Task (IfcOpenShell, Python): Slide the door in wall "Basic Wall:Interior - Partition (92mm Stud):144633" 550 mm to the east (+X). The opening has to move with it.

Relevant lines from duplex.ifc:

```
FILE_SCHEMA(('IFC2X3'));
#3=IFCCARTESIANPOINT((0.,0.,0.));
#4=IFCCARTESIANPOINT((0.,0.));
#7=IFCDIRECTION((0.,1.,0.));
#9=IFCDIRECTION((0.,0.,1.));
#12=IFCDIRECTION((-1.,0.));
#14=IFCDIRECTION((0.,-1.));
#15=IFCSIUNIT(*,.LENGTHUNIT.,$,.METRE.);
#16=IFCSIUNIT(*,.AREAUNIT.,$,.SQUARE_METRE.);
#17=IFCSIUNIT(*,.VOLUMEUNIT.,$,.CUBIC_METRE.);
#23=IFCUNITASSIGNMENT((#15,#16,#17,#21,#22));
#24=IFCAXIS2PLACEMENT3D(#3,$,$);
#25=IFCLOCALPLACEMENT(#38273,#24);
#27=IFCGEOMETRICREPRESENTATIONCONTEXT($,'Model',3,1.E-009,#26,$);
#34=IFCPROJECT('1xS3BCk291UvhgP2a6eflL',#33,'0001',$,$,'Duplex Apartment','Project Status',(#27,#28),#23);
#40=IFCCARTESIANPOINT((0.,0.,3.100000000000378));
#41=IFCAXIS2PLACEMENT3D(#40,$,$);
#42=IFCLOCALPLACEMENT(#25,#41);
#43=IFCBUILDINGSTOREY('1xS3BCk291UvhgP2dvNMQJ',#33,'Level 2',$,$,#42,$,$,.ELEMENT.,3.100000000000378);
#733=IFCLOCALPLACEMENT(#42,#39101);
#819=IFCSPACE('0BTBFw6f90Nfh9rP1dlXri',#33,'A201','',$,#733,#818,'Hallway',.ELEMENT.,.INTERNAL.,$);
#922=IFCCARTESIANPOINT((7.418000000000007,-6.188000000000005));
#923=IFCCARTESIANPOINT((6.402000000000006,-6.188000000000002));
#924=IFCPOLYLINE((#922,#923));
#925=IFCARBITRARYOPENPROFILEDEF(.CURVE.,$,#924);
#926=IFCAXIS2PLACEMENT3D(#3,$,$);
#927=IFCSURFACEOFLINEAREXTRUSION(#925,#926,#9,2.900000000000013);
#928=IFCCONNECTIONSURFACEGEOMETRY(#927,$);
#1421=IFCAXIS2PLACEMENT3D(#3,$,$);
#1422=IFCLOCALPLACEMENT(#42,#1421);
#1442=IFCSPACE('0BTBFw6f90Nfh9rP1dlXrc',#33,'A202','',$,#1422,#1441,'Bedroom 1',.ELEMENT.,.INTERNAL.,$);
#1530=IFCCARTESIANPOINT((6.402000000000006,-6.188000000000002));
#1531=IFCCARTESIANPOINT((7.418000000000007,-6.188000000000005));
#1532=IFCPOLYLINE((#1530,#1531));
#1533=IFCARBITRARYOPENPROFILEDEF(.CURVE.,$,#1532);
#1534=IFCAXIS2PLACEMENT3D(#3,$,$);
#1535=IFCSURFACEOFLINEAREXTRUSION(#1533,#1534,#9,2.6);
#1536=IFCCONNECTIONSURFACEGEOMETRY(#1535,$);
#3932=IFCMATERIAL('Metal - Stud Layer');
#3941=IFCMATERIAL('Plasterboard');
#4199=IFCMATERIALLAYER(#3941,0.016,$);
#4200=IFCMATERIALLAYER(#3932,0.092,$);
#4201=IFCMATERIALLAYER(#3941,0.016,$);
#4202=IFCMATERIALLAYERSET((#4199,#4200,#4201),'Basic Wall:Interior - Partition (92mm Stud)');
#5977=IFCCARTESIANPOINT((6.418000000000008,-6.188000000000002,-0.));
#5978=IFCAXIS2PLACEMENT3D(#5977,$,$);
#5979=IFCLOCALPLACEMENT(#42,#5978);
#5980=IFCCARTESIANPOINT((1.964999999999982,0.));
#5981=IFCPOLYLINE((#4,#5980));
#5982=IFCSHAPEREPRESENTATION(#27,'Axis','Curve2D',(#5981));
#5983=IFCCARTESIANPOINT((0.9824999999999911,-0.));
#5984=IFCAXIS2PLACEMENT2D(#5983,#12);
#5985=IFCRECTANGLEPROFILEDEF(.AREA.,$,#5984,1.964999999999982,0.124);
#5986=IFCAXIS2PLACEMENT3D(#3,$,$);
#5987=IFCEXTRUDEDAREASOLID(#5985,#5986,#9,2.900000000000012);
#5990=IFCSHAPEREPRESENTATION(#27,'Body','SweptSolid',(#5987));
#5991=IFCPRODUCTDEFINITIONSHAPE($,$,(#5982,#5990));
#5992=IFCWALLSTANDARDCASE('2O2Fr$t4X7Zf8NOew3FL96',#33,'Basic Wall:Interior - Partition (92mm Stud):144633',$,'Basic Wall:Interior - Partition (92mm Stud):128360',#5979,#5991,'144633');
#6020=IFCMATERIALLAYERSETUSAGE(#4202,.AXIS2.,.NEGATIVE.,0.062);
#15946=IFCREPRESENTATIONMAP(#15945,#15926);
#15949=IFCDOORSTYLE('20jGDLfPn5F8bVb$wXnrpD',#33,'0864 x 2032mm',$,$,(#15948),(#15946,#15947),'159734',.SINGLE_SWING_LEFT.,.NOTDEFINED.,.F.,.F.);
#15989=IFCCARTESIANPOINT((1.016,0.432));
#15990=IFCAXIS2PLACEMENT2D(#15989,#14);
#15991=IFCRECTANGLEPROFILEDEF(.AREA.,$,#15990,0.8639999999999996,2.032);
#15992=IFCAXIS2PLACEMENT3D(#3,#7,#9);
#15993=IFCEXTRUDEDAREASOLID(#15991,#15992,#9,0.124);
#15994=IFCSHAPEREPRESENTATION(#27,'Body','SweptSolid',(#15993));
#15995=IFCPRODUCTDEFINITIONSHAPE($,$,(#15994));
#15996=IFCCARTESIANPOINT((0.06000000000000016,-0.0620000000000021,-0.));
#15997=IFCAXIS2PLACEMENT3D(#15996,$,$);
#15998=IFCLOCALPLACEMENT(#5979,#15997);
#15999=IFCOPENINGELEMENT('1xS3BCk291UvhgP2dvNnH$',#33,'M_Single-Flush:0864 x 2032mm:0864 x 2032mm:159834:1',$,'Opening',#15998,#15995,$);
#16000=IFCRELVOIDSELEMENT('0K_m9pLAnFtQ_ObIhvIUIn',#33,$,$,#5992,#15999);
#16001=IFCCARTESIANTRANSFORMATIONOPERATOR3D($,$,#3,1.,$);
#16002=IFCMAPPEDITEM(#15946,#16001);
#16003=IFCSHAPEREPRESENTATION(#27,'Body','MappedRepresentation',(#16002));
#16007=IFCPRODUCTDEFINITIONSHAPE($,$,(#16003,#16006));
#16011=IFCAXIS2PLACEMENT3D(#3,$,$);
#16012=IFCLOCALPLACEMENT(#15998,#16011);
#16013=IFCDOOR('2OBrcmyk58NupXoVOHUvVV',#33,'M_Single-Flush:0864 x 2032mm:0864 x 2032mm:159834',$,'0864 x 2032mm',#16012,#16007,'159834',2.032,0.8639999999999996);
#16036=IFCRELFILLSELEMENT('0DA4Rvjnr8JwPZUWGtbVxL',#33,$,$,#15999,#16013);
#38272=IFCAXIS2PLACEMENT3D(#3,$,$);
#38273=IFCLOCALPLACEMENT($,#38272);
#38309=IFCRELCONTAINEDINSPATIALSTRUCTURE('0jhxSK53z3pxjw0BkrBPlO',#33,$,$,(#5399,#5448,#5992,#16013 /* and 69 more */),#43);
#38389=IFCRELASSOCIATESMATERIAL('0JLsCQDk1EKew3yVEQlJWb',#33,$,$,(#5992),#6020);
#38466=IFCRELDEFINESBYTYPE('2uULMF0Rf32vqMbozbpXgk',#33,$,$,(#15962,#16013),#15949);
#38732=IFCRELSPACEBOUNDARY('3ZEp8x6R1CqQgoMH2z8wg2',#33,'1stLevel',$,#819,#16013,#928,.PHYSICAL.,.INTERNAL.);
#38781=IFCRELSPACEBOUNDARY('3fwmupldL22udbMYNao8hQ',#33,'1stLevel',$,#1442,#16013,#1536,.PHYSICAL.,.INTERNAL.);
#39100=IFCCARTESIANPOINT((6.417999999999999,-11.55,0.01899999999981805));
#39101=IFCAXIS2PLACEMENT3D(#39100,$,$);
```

```python
import numpy as np
import ifcopenshell
import ifcopenshell.api.geometry
import ifcopenshell.util.placement
import ifcopenshell.util.unit

model = ifcopenshell.open("duplex.ifc")
unit_scale = ifcopenshell.util.unit.calculate_unit_scale(model)

door = model.by_id(16013)
opening = door.FillsVoids[0].RelatingOpeningElement
wall = opening.VoidsElements[0].RelatingBuildingElement

wall_matrix = ifcopenshell.util.placement.get_local_placement(wall.ObjectPlacement)
shift = wall_matrix[:3, 0] * 0.55 / unit_scale
before = ifcopenshell.util.placement.get_local_placement(door.ObjectPlacement)[:3, 3].copy()

# The door is placed relative to its opening, so it follows when the opening moves.
matrix = ifcopenshell.util.placement.get_local_placement(opening.ObjectPlacement)
matrix[:3, 3] += shift
ifcopenshell.api.geometry.edit_object_placement(
    model, product=opening, matrix=matrix, is_si=False, should_transform_children=True
)

# Space boundary surfaces are stored in each space's coordinates; move them too.
for rel in door.ProvidesBoundaries:
    if not rel.ConnectionGeometry:
        continue
    surface = rel.ConnectionGeometry.SurfaceOnRelatingElement
    space_matrix = ifcopenshell.util.placement.get_local_placement(rel.RelatingSpace.ObjectPlacement)
    point = np.array(surface.Position.Location.Coordinates) + space_matrix[:3, :3].T @ shift
    surface.Position = model.createIfcAxis2Placement3D(
        model.createIfcCartesianPoint(point.tolist()), surface.Position.Axis, surface.Position.RefDirection
    )

after = ifcopenshell.util.placement.get_local_placement(door.ObjectPlacement)[:3, 3]
print("door moved by", (after - before).round(3) + 0.0)

model.write("duplex-out.ifc")
```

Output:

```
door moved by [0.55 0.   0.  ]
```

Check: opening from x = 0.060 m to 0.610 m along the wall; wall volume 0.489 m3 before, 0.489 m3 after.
